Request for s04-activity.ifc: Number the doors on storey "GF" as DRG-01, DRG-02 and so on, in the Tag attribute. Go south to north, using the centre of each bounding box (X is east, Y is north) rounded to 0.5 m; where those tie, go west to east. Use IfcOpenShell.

First a look at what the model holds.

```python
import ifcopenshell
import ifcopenshell.util.element
import ifcopenshell.util.placement

model = ifcopenshell.open("s04-activity.ifc")
print(model.schema)
storey = next(s for s in model.by_type("IfcBuildingStorey") if s.Name == "GF")
doors = [e for e in ifcopenshell.util.element.get_decomposition(storey) if e.is_a("IfcDoor")]
for e in sorted(doors, key=lambda e: e.id()):
    origin = ifcopenshell.util.placement.get_local_placement(e.ObjectPlacement)[:3, 3]
    print(e.id(), e.Tag, e.Name, origin.round(2) + 0.0, sep=" | ")
```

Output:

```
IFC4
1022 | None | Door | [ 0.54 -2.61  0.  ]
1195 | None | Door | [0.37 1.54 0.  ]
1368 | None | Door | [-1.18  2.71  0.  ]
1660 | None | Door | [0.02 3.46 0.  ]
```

```python
import ifcopenshell
import ifcopenshell.geom
import ifcopenshell.util.element
import ifcopenshell.util.shape

model = ifcopenshell.open("s04-activity.ifc")
settings = ifcopenshell.geom.settings()
settings.set("use-world-coords", True)


def centre(element):
    shape = ifcopenshell.geom.create_shape(settings, element)
    return ifcopenshell.util.shape.get_bbox_centroid(shape.geometry)


storey = next(s for s in model.by_type("IfcBuildingStorey") if s.Name == "GF")
doors = [e for e in ifcopenshell.util.element.get_decomposition(storey) if e.is_a("IfcDoor")]

# Insertion points can sit at a corner or the storey origin, so sort by the geometry (in metres).
centres = {e: centre(e) for e in doors}
doors.sort(key=lambda e: (round(centres[e][1] / 0.5), centres[e][0]))

for i, e in enumerate(doors, start=1):
    number = f"DRG-{i:02d}"
    e.Tag = number
    print(e.id(), number)

model.write("s04-activity_updated.ifc")
```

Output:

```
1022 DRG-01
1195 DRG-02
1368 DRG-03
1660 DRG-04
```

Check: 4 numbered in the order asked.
